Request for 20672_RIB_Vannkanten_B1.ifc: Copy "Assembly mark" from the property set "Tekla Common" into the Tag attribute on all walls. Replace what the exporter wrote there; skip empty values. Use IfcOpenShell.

First a look at what the model holds.

```python
import ifcopenshell
import ifcopenshell.util.element

model = ifcopenshell.open("20672_RIB_Vannkanten_B1.ifc")
print(model.schema)
walls = model.by_type("IfcWall")
print(len(walls), "walls")
for e in walls[:8]:
    source = ifcopenshell.util.element.get_pset(e, "Tekla Common", "Assembly mark")
    target = e.Tag
    print(e.id(), repr(source), repr(target), sep=" | ")
```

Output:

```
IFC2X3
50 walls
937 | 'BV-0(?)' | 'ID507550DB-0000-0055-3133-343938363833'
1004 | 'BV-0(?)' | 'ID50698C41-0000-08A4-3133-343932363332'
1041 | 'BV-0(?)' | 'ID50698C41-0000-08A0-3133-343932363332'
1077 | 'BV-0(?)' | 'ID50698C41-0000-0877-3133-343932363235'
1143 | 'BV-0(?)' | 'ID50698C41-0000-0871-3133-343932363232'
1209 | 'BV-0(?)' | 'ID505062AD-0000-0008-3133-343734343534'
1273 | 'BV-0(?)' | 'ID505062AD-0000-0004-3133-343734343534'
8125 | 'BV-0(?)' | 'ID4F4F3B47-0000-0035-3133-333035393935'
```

```python
import ifcopenshell
import ifcopenshell.util.element

model = ifcopenshell.open("20672_RIB_Vannkanten_B1.ifc")

count = 0
for e in model.by_type("IfcWall"):
    value = ifcopenshell.util.element.get_pset(e, "Tekla Common", "Assembly mark")
    current = e.Tag
    if not value or not value.strip() or current == value:
        continue
    e.Tag = value
    count += 1

print(count, "walls updated")

model.write("20672_RIB_Vannkanten_B1_v2.ifc")
```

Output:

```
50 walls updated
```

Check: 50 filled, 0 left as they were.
